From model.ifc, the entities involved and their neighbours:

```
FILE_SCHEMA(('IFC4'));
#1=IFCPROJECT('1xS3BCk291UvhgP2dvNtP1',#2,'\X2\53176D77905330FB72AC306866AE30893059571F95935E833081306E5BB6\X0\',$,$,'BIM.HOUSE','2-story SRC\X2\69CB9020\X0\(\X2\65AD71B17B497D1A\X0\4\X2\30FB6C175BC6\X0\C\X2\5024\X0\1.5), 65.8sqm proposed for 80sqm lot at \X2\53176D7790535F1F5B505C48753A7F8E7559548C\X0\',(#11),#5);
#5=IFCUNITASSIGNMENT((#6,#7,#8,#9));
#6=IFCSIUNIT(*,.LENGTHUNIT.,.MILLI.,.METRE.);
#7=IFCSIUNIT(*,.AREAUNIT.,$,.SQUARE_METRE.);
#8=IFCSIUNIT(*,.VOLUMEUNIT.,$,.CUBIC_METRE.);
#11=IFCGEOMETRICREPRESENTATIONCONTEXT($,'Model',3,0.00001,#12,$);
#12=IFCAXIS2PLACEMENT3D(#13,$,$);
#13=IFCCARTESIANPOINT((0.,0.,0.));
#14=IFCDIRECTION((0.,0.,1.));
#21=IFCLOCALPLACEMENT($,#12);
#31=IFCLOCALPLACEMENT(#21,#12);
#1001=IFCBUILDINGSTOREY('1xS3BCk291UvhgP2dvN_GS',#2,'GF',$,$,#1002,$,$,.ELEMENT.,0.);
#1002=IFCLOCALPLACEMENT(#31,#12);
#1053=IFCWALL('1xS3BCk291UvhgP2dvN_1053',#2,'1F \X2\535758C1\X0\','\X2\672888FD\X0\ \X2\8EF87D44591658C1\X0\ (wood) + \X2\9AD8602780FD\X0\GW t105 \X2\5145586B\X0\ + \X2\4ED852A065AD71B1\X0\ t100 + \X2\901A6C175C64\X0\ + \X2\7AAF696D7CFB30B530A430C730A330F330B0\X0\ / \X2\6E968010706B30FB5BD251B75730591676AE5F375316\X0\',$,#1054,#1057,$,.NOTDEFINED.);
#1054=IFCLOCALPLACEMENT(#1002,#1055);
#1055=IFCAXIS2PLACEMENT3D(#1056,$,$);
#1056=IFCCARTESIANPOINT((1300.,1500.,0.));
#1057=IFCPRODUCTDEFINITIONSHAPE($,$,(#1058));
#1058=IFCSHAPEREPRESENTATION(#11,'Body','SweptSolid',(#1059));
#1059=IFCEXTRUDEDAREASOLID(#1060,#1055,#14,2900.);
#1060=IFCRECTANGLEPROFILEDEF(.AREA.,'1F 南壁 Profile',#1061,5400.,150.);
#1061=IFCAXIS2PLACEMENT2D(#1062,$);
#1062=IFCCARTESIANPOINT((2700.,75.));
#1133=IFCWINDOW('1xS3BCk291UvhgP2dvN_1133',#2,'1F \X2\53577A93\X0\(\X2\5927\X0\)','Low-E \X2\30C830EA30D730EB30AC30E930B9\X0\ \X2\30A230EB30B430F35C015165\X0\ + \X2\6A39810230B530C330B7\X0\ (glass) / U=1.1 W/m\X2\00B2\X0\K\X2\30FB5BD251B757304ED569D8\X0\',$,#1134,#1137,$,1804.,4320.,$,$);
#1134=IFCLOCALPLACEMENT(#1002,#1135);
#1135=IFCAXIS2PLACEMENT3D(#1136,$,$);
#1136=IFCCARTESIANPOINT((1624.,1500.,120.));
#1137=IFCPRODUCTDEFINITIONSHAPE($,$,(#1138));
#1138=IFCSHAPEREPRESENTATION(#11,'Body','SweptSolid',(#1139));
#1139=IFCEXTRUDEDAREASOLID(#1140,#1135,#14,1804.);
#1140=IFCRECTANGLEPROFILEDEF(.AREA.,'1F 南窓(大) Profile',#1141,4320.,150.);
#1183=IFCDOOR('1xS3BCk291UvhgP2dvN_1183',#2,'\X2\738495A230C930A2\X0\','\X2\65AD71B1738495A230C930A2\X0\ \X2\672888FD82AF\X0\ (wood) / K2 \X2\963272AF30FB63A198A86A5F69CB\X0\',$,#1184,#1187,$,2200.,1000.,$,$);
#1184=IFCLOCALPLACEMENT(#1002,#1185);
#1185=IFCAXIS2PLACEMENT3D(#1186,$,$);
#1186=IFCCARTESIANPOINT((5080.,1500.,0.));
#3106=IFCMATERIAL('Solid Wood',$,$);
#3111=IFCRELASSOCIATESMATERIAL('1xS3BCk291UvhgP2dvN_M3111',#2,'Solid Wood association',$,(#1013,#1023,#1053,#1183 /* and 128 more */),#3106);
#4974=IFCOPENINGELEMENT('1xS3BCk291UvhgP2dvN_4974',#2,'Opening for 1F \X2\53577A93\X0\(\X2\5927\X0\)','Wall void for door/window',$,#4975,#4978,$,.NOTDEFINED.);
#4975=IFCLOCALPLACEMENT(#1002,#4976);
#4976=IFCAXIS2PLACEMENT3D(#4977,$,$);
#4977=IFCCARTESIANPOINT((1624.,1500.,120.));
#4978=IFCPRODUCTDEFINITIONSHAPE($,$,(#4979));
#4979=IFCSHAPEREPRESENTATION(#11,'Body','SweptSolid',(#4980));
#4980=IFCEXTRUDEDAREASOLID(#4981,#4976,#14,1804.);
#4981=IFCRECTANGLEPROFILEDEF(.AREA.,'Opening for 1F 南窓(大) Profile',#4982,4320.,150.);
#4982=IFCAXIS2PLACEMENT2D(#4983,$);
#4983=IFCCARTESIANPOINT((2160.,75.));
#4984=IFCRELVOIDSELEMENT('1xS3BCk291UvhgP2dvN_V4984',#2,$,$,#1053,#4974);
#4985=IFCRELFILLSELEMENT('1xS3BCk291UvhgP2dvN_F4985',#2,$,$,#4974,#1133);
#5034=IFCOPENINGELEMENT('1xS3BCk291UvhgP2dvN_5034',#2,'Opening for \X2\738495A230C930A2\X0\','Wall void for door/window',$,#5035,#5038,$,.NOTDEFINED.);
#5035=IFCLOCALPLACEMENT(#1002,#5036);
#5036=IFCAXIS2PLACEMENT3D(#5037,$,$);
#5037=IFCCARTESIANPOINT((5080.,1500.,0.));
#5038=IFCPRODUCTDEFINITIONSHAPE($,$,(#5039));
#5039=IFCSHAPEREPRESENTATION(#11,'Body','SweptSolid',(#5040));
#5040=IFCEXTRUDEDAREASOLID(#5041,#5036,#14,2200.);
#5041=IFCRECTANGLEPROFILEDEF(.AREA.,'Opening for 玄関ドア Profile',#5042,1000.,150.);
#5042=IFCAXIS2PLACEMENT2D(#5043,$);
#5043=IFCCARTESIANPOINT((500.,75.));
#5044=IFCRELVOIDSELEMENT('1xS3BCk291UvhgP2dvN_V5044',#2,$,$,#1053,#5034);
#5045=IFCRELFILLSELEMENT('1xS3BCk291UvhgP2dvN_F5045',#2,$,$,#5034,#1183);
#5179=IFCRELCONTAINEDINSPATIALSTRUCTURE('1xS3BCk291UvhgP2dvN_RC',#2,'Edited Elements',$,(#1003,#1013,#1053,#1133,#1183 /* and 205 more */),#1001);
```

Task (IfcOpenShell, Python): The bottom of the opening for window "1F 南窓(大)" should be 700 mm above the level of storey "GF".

```python
import numpy as np
import ifcopenshell
import ifcopenshell.api.geometry
import ifcopenshell.geom
import ifcopenshell.util.element
import ifcopenshell.util.placement
import ifcopenshell.util.shape
import ifcopenshell.util.unit

model = ifcopenshell.open("model.ifc")
unit_scale = ifcopenshell.util.unit.calculate_unit_scale(model)

window = model.by_id(1133)
opening = window.FillsVoids[0].RelatingOpeningElement
storey = ifcopenshell.util.element.get_container(window, ifc_class="IfcBuildingStorey")
level = ifcopenshell.util.placement.get_local_placement(storey.ObjectPlacement)[2, 3]

# The opening's origin need not be at the sill, so measure its lowest point.
shape = ifcopenshell.geom.create_shape(ifcopenshell.geom.settings(), opening)
bottom = ifcopenshell.util.shape.get_shape_bottom_elevation(shape, shape.geometry) / unit_scale
dz = level + 700.0 - bottom

shift = np.array([0.0, 0.0, dz])
# The window is not placed relative to its opening, so move both.
for product in (opening, window):
    matrix = ifcopenshell.util.placement.get_local_placement(product.ObjectPlacement)
    matrix[:3, 3] += shift
    ifcopenshell.api.geometry.edit_object_placement(model, product=product, matrix=matrix, is_si=False)

print(f"moved by {dz * unit_scale:+.3f} m")

model.write("model-out.ifc")
```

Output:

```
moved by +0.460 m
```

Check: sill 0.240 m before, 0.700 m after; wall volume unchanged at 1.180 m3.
